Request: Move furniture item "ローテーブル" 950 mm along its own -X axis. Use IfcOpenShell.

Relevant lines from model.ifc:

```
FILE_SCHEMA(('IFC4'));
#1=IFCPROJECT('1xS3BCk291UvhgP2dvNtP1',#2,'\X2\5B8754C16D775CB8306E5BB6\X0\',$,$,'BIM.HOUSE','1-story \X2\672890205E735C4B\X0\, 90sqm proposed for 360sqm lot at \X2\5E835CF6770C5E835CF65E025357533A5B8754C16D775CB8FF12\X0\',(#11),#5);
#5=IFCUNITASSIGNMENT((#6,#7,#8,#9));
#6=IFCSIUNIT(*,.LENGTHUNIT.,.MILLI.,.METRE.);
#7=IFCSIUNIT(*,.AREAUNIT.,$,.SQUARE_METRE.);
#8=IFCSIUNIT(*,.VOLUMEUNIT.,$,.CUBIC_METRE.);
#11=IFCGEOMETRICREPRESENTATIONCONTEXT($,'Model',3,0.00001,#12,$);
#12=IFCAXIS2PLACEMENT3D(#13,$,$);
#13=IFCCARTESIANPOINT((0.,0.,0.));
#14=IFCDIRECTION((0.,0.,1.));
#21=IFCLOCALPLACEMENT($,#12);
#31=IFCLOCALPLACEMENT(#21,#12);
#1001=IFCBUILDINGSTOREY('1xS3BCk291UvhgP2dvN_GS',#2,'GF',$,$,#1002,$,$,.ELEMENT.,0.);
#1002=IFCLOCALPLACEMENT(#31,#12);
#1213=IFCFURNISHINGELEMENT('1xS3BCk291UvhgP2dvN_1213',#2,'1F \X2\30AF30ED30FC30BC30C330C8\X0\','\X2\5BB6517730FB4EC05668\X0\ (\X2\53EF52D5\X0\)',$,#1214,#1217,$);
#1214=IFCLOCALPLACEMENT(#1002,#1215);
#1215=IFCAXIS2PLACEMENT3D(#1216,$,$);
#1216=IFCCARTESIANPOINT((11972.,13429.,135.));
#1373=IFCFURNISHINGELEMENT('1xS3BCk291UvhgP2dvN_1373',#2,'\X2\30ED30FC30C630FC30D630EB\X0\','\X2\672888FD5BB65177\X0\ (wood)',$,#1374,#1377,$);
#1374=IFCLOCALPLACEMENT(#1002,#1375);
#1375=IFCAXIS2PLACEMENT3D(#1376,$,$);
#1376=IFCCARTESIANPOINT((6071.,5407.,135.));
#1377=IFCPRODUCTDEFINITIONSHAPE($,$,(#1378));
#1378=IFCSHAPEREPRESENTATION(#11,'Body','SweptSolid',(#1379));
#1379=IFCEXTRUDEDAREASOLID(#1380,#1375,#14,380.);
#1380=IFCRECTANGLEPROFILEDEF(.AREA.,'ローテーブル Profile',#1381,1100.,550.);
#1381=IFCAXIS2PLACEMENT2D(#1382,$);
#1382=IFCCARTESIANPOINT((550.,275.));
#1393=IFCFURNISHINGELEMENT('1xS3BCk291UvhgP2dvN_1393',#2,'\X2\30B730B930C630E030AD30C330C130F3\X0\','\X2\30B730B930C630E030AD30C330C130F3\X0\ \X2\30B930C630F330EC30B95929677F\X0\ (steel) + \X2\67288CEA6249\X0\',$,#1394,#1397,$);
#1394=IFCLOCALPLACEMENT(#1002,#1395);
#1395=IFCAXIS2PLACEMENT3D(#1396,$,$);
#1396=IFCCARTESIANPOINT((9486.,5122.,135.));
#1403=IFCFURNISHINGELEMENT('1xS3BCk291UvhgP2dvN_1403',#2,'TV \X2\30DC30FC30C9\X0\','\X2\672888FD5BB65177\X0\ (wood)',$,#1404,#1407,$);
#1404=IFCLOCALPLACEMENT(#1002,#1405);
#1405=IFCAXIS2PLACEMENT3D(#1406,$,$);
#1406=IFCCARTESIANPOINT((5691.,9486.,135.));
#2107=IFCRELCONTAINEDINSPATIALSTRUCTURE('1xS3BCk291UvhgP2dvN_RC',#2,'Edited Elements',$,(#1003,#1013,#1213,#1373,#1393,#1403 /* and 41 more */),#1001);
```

```python
import ifcopenshell
import ifcopenshell.api.geometry
import ifcopenshell.util.placement
import ifcopenshell.util.unit

model = ifcopenshell.open("model.ifc")
unit_scale = ifcopenshell.util.unit.calculate_unit_scale(model)

item = model.by_guid("1xS3BCk291UvhgP2dvN_1373")
matrix = ifcopenshell.util.placement.get_local_placement(item.ObjectPlacement)
matrix[:3, 3] -= matrix[:3, 0] * 0.95 / unit_scale
ifcopenshell.api.geometry.edit_object_placement(model, product=item, matrix=matrix, is_si=False)

print(ifcopenshell.util.placement.get_local_placement(item.ObjectPlacement).round(3) + 0.0)

model.write("model_edited.ifc")
```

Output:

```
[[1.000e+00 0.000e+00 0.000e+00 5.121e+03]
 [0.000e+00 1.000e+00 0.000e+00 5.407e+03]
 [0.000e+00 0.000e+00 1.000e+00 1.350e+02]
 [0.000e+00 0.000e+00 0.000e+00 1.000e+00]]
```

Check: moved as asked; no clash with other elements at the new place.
